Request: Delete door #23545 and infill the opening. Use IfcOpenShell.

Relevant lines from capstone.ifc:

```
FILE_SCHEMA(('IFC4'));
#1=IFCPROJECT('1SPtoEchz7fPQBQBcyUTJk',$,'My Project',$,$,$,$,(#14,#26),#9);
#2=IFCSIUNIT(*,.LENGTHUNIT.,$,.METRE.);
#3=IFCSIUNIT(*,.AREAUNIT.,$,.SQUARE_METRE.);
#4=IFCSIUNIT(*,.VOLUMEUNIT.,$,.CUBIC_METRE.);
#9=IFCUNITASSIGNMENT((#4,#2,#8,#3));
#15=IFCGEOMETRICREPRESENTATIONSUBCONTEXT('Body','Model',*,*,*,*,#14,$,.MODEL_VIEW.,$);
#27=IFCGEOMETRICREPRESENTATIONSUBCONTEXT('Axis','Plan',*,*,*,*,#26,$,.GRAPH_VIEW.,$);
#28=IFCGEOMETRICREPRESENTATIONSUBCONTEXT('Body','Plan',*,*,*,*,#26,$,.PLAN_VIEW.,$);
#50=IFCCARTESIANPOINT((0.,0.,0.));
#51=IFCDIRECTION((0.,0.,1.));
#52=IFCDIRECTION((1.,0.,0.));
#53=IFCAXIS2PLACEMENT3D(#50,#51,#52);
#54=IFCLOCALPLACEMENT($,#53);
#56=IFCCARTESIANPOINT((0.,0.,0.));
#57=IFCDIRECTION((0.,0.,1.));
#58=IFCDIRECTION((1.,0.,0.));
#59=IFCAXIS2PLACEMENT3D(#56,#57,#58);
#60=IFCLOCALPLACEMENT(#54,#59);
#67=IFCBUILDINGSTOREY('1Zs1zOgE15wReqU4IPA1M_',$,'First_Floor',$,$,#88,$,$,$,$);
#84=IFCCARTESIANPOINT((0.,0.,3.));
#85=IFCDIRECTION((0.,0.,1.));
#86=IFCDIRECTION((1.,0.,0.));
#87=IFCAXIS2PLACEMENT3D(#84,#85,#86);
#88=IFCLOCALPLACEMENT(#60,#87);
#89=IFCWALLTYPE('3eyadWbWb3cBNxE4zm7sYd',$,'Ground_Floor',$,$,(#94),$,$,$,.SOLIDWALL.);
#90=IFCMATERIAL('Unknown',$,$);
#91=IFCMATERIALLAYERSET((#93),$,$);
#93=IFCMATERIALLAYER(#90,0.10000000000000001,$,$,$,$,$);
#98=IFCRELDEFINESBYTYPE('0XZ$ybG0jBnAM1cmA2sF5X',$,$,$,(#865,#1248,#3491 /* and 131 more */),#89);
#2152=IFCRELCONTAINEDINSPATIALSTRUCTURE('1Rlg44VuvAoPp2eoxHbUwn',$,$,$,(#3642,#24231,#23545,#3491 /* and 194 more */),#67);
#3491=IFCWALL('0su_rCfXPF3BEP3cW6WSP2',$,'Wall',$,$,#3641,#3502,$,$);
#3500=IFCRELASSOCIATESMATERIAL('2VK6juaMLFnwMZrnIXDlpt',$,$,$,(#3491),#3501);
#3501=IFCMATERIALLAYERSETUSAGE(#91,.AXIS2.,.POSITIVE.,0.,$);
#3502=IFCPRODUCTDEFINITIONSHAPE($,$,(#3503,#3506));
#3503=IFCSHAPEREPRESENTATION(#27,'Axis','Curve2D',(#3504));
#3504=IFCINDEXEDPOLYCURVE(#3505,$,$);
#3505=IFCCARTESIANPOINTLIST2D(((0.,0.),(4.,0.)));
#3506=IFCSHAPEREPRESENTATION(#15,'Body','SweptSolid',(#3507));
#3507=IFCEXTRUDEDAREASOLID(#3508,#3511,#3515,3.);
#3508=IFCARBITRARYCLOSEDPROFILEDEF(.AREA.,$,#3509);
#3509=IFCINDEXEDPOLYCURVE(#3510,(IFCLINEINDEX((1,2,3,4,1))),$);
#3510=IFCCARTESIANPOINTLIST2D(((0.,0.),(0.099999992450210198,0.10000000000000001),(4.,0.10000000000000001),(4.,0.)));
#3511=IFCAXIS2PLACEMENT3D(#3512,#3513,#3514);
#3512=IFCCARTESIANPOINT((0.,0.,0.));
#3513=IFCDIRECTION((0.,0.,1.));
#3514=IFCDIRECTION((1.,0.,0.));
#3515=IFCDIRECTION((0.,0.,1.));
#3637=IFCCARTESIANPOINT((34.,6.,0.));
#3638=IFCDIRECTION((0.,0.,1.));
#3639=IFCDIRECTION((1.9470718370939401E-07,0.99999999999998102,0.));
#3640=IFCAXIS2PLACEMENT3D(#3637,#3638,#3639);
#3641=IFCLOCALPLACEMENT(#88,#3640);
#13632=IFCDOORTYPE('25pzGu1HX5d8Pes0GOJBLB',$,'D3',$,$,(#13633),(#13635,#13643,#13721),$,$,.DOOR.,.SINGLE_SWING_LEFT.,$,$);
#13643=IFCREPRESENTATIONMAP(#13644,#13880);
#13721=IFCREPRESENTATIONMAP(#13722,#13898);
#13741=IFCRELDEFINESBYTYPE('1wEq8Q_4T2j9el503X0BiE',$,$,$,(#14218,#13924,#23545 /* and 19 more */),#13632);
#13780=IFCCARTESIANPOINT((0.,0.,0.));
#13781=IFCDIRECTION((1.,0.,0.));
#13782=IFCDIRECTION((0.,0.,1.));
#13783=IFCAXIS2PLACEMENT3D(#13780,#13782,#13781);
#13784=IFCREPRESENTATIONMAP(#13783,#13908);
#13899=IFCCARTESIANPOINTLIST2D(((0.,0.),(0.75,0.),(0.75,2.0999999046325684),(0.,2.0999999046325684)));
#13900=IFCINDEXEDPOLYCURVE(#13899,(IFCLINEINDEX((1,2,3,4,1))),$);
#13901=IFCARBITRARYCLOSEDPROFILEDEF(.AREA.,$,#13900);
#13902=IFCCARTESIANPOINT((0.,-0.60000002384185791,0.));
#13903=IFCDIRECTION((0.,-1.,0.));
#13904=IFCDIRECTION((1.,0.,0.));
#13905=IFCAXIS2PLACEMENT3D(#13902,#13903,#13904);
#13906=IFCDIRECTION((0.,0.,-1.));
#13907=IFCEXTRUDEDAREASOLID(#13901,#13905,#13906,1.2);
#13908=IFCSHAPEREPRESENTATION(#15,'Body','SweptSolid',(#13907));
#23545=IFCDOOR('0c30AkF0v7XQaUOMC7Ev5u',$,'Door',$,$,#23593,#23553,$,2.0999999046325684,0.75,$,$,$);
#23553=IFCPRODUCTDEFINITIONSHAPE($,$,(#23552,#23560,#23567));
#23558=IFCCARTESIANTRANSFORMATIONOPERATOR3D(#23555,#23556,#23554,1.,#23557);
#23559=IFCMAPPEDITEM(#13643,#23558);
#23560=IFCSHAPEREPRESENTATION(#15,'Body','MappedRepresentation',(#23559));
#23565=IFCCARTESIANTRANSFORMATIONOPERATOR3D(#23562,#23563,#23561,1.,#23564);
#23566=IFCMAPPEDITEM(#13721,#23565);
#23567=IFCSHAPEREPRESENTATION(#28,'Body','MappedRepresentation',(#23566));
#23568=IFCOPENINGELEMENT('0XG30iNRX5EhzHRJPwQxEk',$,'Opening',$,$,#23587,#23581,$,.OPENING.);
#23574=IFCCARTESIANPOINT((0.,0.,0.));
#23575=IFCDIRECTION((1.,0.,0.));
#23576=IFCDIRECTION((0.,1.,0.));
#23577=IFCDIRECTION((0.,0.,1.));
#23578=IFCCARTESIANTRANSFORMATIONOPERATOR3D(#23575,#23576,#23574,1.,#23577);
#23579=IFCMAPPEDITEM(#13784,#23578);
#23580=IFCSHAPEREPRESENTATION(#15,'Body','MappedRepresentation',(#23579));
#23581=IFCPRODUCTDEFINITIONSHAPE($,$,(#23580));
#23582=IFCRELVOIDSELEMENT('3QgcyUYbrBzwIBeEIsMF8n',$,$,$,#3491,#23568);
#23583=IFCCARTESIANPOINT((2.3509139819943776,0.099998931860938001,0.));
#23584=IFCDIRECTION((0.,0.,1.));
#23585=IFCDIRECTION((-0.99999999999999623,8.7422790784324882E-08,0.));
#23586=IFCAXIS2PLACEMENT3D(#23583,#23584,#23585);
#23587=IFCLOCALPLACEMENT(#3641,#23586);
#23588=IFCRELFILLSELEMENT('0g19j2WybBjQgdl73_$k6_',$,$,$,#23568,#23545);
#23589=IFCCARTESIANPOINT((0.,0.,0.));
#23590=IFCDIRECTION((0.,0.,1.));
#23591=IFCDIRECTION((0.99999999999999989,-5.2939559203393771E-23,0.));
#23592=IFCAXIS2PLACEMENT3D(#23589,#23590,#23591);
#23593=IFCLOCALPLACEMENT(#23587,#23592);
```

```python
import ifcopenshell
import ifcopenshell.api.feature
import ifcopenshell.api.root
import ifcopenshell.geom
import ifcopenshell.util.shape

model = ifcopenshell.open("capstone.ifc")
settings = ifcopenshell.geom.settings()


def volume(element):
    """Net volume in cubic metres, openings subtracted."""
    shape = ifcopenshell.geom.create_shape(settings, element)
    return ifcopenshell.util.shape.get_volume(shape.geometry)


door = model.by_guid("0c30AkF0v7XQaUOMC7Ev5u")
opening = door.FillsVoids[0].RelatingOpeningElement
wall = opening.VoidsElements[0].RelatingBuildingElement
before = volume(wall)

ifcopenshell.api.root.remove_product(model, product=door)
ifcopenshell.api.feature.remove_feature(model, feature=opening)

after = volume(wall)

print(f"wall volume {before:.3f} -> {after:.3f} m3")

model.write("capstone_edited.ifc")
```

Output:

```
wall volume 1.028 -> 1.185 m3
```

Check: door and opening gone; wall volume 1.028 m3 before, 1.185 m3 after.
